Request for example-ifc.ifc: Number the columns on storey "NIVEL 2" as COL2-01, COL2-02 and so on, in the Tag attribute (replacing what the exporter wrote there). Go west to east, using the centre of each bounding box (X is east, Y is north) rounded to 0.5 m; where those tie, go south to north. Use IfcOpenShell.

First a look at what the model holds.

```python
import ifcopenshell
import ifcopenshell.util.element
import ifcopenshell.util.placement

model = ifcopenshell.open("example-ifc.ifc")
print(model.schema)
storey = next(s for s in model.by_type("IfcBuildingStorey") if s.Name == "NIVEL 2")
columns = [e for e in ifcopenshell.util.element.get_decomposition(storey) if e.is_a("IfcColumn")]
for e in sorted(columns, key=lambda e: e.id()):
    origin = ifcopenshell.util.placement.get_local_placement(e.ObjectPlacement)[:3, 3]
    print(e.id(), e.Tag, e.Name, origin.round(2) + 0.0, sep=" | ")
```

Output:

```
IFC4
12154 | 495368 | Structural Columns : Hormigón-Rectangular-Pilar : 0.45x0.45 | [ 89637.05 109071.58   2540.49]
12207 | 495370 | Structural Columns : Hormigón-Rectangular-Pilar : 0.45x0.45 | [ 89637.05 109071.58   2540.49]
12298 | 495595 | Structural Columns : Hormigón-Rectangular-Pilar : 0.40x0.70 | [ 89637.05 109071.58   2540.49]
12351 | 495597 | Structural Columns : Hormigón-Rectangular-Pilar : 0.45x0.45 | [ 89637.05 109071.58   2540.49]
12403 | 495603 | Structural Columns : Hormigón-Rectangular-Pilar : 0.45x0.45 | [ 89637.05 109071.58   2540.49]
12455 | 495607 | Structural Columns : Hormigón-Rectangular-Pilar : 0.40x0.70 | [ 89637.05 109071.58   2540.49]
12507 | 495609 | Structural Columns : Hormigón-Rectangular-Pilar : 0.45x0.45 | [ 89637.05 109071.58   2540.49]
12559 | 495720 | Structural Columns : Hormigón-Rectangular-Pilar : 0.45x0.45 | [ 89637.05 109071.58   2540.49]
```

```python
import ifcopenshell
import ifcopenshell.geom
import ifcopenshell.util.element
import ifcopenshell.util.shape

model = ifcopenshell.open("example-ifc.ifc")
settings = ifcopenshell.geom.settings()
settings.set("use-world-coords", True)


def centre(element):
    shape = ifcopenshell.geom.create_shape(settings, element)
    return ifcopenshell.util.shape.get_bbox_centroid(shape.geometry)


storey = next(s for s in model.by_type("IfcBuildingStorey") if s.Name == "NIVEL 2")
columns = [e for e in ifcopenshell.util.element.get_decomposition(storey) if e.is_a("IfcColumn")]

# Insertion points can sit at a corner or the storey origin, so sort by the geometry (in metres).
centres = {e: centre(e) for e in columns}
columns.sort(key=lambda e: (round(centres[e][0] / 0.5), centres[e][1]))

for i, e in enumerate(columns, start=1):
    number = f"COL2-{i:02d}"
    e.Tag = number
    print(e.id(), number)

model.write("example-ifc_edited.ifc")
```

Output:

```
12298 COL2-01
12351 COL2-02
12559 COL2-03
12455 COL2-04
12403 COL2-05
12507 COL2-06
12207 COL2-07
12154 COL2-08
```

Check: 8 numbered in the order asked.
